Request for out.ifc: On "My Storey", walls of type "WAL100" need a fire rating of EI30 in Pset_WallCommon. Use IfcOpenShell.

First a look at what the model holds.

```python
import ifcopenshell
import ifcopenshell.util.element

model = ifcopenshell.open("out.ifc")
print(model.schema)
storey = next(s for s in model.by_type("IfcBuildingStorey") if s.Name == "My Storey")
walls = [e for e in ifcopenshell.util.element.get_decomposition(storey) if e.is_a("IfcWall")]
seen = {}
for e in walls:
    element_type = ifcopenshell.util.element.get_type(e)
    key = (element_type.Name if element_type != e and element_type else None, ifcopenshell.util.element.get_pset(e, "Pset_WallCommon", "FireRating"))
    seen[key] = seen.get(key, 0) + 1
for (name, value), count in sorted(seen.items(), key=str):
    print(count, "x", name, "|", value)
```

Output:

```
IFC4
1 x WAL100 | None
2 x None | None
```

```python
import ifcopenshell
import ifcopenshell.api.pset
import ifcopenshell.util.element

model = ifcopenshell.open("out.ifc")

storey = next(s for s in model.by_type("IfcBuildingStorey") if s.Name == "My Storey")
walls = [e for e in ifcopenshell.util.element.get_decomposition(storey) if e.is_a("IfcWall")]

count = 0
for e in walls:
    element_type = ifcopenshell.util.element.get_type(e)
    if element_type in (None, e) or element_type.Name != "WAL100":
        continue
    # add_pset returns the element's existing set when there is one.
    pset = ifcopenshell.api.pset.add_pset(model, product=e, name="Pset_WallCommon")
    ifcopenshell.api.pset.edit_pset(model, pset=pset, properties={"FireRating": "EI30"})
    count += 1

print(count, "walls updated")

model.write("out_edited.ifc")
```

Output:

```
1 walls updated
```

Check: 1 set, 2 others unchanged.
